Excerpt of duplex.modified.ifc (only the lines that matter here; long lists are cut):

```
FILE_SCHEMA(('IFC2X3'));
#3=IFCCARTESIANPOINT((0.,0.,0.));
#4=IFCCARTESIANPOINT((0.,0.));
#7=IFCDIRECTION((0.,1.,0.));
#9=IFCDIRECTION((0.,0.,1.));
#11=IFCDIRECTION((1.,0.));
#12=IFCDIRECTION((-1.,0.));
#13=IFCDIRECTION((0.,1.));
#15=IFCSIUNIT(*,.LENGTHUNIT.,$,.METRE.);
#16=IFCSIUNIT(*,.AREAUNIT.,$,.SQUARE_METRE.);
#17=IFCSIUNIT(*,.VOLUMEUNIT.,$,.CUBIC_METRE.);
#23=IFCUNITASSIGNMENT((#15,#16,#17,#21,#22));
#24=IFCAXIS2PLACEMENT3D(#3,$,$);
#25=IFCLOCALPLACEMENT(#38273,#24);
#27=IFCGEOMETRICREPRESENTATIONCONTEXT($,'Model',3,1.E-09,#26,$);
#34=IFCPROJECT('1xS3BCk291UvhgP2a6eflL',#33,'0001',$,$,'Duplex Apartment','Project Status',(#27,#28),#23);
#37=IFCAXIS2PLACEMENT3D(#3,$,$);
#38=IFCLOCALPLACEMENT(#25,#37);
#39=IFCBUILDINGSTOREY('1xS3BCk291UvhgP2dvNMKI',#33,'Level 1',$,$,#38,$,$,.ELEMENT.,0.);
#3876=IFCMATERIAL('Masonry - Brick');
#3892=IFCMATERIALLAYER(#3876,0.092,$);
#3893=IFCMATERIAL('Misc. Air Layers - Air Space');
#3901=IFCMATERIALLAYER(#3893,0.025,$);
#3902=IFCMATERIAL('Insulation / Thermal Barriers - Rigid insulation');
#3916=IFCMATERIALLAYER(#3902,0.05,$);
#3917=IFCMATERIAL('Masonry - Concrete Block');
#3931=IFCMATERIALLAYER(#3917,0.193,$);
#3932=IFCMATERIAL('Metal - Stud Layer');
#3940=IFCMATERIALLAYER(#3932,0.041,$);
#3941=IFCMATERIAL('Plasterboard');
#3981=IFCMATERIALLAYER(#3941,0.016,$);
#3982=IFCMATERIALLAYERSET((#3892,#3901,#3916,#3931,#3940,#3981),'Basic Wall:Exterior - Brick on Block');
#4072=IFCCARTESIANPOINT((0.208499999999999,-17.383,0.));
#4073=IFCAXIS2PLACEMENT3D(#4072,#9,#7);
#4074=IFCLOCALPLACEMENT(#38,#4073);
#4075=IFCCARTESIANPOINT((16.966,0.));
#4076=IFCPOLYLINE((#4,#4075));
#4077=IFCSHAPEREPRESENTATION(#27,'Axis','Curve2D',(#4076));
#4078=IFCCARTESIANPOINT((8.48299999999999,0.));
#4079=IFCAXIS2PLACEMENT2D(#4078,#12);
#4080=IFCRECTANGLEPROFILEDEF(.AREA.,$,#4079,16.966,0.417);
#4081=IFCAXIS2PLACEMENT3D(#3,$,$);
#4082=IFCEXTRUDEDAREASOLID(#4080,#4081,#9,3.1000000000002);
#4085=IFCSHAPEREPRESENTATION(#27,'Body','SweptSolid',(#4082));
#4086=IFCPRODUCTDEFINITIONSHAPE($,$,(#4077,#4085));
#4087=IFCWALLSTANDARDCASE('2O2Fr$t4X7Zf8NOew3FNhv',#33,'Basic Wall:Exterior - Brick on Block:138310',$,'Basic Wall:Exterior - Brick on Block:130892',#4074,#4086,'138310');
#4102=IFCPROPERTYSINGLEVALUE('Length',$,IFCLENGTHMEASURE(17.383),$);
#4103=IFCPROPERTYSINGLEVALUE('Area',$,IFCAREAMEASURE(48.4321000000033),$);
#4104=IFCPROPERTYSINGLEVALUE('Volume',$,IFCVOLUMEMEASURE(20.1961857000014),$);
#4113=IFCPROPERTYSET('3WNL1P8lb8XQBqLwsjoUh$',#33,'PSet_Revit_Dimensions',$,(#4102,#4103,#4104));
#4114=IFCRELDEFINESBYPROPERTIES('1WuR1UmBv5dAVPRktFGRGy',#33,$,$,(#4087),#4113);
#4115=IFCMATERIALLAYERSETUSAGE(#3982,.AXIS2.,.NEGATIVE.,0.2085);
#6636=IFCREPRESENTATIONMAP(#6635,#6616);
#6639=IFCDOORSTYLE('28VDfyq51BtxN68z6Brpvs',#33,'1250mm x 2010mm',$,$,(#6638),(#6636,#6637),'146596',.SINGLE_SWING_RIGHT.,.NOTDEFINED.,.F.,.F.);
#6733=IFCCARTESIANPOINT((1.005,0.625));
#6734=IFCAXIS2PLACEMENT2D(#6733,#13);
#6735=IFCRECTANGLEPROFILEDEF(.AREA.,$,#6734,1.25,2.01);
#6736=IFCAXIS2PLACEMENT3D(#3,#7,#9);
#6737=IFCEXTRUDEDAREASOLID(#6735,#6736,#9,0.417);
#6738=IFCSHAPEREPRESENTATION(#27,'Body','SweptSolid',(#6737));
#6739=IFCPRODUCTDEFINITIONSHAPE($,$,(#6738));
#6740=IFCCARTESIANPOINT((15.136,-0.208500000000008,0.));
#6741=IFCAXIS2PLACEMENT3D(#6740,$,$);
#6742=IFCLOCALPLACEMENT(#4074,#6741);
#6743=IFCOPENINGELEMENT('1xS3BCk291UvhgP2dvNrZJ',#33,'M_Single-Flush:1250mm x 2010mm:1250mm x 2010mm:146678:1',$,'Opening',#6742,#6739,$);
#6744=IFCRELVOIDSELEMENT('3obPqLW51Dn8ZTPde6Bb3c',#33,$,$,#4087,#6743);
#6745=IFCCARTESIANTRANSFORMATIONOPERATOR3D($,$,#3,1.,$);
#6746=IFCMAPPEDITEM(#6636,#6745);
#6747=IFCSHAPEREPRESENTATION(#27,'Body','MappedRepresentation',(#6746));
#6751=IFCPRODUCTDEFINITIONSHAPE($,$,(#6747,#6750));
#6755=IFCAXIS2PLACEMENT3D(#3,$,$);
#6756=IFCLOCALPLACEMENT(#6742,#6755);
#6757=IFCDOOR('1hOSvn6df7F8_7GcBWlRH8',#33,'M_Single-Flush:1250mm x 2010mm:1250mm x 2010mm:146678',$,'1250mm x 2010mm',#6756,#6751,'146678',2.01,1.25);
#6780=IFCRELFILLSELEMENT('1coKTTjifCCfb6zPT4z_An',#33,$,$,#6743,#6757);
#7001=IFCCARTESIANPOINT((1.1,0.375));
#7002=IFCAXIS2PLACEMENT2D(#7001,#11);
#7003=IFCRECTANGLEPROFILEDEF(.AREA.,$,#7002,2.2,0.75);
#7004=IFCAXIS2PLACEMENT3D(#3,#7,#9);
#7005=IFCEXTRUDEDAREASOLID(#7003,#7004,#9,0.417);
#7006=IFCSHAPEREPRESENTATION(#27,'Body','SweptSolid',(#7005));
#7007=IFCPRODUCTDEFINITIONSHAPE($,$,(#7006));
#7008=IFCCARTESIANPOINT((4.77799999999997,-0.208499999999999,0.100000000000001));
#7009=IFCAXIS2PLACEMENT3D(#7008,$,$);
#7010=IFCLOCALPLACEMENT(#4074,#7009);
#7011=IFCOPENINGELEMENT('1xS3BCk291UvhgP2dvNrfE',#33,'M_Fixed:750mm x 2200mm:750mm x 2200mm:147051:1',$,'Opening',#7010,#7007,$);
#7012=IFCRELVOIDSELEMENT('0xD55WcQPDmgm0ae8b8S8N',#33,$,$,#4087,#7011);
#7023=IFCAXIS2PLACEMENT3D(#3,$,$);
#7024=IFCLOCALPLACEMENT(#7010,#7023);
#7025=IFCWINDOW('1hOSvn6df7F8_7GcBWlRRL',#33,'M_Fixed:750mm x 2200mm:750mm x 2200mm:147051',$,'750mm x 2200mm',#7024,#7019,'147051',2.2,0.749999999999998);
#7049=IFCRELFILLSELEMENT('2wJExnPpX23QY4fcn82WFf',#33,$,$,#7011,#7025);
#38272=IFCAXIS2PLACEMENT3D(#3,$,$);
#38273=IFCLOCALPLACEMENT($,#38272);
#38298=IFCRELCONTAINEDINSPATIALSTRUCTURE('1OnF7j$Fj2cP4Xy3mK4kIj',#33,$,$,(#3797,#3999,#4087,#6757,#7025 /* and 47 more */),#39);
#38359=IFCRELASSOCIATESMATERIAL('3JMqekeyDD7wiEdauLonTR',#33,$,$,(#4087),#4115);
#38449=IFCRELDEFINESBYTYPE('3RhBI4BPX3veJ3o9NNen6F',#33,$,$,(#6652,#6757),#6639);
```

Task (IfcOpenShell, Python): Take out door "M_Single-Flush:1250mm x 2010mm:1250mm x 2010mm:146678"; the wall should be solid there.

```python
import ifcopenshell
import ifcopenshell.api.feature
import ifcopenshell.api.pset
import ifcopenshell.api.root
import ifcopenshell.geom
import ifcopenshell.util.element
import ifcopenshell.util.shape
import ifcopenshell.util.unit

model = ifcopenshell.open("duplex.modified.ifc")
area_scale = ifcopenshell.util.unit.calculate_unit_scale(model, "AREAUNIT")
volume_scale = ifcopenshell.util.unit.calculate_unit_scale(model, "VOLUMEUNIT")
settings = ifcopenshell.geom.settings()


def volume(element):
    """Net volume in cubic metres, openings subtracted."""
    shape = ifcopenshell.geom.create_shape(settings, element)
    return ifcopenshell.util.shape.get_volume(shape.geometry)


door = model.by_guid("1hOSvn6df7F8_7GcBWlRH8")
opening = door.FillsVoids[0].RelatingOpeningElement
wall = opening.VoidsElements[0].RelatingBuildingElement
before = volume(wall)

ifcopenshell.api.root.remove_product(model, product=door)
ifcopenshell.api.feature.remove_feature(model, feature=opening)

after = volume(wall)
thickness = 0.417  # wall thickness in metres

# Update the wall's stored quantities.
pset = model.by_id(ifcopenshell.util.element.get_pset(wall, "PSet_Revit_Dimensions", should_inherit=False)["id"])
ifcopenshell.api.pset.edit_pset(model, pset=pset, properties={
    "Area": model.create_entity("IfcAreaMeasure", after / thickness / area_scale),
    "Volume": model.create_entity("IfcVolumeMeasure", after / volume_scale),
})

print(f"wall volume {before:.3f} -> {after:.3f} m3")

model.write("duplex.modified_v2.ifc")
```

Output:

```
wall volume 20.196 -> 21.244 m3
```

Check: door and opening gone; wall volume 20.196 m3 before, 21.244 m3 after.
